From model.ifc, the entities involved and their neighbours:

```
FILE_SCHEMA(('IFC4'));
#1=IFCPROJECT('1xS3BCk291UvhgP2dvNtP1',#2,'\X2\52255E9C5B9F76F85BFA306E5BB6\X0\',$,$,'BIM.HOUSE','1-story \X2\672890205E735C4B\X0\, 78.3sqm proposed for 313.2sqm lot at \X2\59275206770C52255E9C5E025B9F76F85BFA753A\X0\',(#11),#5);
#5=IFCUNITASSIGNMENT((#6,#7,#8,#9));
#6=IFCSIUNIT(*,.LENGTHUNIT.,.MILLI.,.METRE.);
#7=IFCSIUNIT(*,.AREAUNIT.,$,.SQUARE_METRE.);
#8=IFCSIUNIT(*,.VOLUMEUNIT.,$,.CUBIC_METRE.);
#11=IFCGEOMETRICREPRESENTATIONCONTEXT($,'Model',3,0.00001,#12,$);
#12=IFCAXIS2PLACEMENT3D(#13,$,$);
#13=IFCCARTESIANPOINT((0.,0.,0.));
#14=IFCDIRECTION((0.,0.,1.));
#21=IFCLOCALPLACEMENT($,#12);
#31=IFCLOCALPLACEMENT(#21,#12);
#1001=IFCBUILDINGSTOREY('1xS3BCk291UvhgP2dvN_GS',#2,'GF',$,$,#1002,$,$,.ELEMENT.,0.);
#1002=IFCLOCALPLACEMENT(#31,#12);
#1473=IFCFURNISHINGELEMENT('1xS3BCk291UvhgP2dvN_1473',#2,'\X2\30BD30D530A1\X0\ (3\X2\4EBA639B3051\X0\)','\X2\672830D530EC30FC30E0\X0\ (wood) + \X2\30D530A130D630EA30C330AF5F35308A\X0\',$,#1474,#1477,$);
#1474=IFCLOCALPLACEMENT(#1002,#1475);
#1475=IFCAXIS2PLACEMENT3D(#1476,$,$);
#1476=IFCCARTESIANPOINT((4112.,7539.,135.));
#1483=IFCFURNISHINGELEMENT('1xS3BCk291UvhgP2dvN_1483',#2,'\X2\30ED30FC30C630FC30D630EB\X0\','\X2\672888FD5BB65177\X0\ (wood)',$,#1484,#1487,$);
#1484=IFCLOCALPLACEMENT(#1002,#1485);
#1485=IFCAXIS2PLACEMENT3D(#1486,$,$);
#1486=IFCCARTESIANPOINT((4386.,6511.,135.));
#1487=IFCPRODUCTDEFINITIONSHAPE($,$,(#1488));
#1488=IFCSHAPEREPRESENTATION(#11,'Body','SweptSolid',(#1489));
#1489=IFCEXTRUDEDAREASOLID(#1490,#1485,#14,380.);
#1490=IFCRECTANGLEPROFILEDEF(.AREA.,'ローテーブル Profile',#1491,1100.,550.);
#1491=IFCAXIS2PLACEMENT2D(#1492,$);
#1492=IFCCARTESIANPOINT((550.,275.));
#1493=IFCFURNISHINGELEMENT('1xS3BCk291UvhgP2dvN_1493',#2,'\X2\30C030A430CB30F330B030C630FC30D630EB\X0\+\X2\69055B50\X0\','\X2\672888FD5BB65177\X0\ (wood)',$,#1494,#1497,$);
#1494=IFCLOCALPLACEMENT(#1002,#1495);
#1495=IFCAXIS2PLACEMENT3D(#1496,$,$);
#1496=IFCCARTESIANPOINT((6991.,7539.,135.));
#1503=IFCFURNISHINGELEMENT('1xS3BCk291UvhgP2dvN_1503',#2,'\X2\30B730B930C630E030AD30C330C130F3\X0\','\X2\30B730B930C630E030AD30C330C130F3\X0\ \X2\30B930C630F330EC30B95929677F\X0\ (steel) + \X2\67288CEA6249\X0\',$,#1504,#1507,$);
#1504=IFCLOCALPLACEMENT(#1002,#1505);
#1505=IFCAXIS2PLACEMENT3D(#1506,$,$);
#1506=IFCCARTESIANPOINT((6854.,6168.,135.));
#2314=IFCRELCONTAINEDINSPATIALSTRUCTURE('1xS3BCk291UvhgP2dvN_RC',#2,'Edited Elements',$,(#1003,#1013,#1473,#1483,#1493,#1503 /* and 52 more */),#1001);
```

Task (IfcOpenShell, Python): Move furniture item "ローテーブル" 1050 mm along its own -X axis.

```python
import ifcopenshell
import ifcopenshell.api.geometry
import ifcopenshell.util.placement

model = ifcopenshell.open("model.ifc")

item = model.by_guid("1xS3BCk291UvhgP2dvN_1483")
matrix = ifcopenshell.util.placement.get_local_placement(item.ObjectPlacement)
matrix[:3, 3] -= matrix[:3, 0] * 1050.0
ifcopenshell.api.geometry.edit_object_placement(model, product=item, matrix=matrix, is_si=False)

print(ifcopenshell.util.placement.get_local_placement(item.ObjectPlacement).round(3) + 0.0)

model.write("model_rev.ifc")
```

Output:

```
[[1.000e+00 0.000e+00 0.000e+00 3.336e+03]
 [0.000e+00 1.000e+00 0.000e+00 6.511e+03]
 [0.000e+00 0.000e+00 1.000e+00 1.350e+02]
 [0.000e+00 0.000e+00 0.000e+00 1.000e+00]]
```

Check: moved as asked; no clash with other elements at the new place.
